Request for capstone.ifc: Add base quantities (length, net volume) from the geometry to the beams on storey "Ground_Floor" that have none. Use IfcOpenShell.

First a look at what the model holds.

```python
import ifcopenshell
import ifcopenshell.util.element
import ifcopenshell.util.unit

model = ifcopenshell.open("capstone.ifc")
print(model.schema)
for unit_type in ("LENGTHUNIT", "AREAUNIT", "VOLUMEUNIT"):
    print(unit_type, ifcopenshell.util.unit.calculate_unit_scale(model, unit_type))
storey = next(s for s in model.by_type("IfcBuildingStorey") if s.Name == "Ground_Floor")
beams = [e for e in ifcopenshell.util.element.get_decomposition(storey) if e.is_a("IfcBeam")]
for e in sorted(beams, key=lambda e: e.id()):
    print(e.id(), e.is_a(), e.Name, list(ifcopenshell.util.element.get_psets(e, qtos_only=True)), sep=" | ")
```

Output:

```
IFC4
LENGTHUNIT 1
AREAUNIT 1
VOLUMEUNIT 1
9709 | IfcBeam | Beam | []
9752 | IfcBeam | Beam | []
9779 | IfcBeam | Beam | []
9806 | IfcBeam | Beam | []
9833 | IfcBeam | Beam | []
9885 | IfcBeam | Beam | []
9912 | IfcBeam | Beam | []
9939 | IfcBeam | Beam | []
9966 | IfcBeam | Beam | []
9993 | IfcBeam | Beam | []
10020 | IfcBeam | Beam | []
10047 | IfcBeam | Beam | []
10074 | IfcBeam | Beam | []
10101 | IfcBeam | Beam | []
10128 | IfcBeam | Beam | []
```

```python
import ifcopenshell
import ifcopenshell.api.pset
import ifcopenshell.geom
import ifcopenshell.util.element
import ifcopenshell.util.shape
import ifcopenshell.util.unit

model = ifcopenshell.open("capstone.ifc")
unit_scale = ifcopenshell.util.unit.calculate_unit_scale(model)
volume_scale = ifcopenshell.util.unit.calculate_unit_scale(model, "VOLUMEUNIT")
settings = ifcopenshell.geom.settings()

storey = next(s for s in model.by_type("IfcBuildingStorey") if s.Name == "Ground_Floor")
beams = [e for e in ifcopenshell.util.element.get_decomposition(storey) if e.is_a("IfcBeam")]

for e in sorted(beams, key=lambda e: e.id()):
    if ifcopenshell.util.element.get_psets(e, qtos_only=True, should_inherit=False):
        continue
    # Geometry comes back in metres, in the element's own axes.
    shape = ifcopenshell.geom.create_shape(settings, e)
    values = {
        "Length": ifcopenshell.util.shape.get_max_xyz(shape.geometry) / unit_scale,
        "NetVolume": ifcopenshell.util.shape.get_volume(shape.geometry) / volume_scale,
    }
    qto = ifcopenshell.api.pset.add_qto(model, product=e, name="Qto_BeamBaseQuantities")
    ifcopenshell.api.pset.edit_qto(model, qto=qto, properties=values)
    print(e.id(), {k: round(v, 3) for k, v in values.items()})

model.write("capstone_edited.ifc")
```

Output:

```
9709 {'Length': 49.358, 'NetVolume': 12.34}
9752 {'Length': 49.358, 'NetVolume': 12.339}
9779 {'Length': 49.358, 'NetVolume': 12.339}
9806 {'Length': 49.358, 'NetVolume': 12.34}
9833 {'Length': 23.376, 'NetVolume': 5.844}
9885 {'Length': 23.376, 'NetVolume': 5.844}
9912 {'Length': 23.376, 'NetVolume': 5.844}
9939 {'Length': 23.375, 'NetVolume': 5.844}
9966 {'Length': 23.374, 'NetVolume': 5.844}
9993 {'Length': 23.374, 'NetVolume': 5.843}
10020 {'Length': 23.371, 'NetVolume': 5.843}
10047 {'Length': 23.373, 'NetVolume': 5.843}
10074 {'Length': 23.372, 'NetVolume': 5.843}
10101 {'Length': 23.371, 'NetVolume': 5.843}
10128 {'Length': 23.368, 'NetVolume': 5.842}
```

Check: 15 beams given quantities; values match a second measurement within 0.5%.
